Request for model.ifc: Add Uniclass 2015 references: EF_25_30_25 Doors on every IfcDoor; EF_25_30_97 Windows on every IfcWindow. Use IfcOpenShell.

First a look at what the model holds.

```python
import ifcopenshell

model = ifcopenshell.open("model.ifc")
print(model.schema)
print("classifications:", [c.Name for c in model.by_type("IfcClassification")])
for ifc_class in ("IfcDoor", "IfcRoof", "IfcStair", "IfcWall", "IfcWindow"):
    print(ifc_class, len(model.by_type(ifc_class)))
```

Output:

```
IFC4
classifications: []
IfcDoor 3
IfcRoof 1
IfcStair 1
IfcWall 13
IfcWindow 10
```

```python
import ifcopenshell
import ifcopenshell.api.classification

model = ifcopenshell.open("model.ifc")

system = ifcopenshell.api.classification.add_classification(model, classification="Uniclass 2015")

codes = {
    "IfcDoor": ("EF_25_30_25", "Doors"),
    "IfcWindow": ("EF_25_30_97", "Windows"),
}
for ifc_class, (code, name) in codes.items():
    products = model.by_type(ifc_class)
    ifcopenshell.api.classification.add_reference(
        model, products=products, classification=system, identification=code, name=name
    )
    print(code, len(products))

model.write("model_edited.ifc")
```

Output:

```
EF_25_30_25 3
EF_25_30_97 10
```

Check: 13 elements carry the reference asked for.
